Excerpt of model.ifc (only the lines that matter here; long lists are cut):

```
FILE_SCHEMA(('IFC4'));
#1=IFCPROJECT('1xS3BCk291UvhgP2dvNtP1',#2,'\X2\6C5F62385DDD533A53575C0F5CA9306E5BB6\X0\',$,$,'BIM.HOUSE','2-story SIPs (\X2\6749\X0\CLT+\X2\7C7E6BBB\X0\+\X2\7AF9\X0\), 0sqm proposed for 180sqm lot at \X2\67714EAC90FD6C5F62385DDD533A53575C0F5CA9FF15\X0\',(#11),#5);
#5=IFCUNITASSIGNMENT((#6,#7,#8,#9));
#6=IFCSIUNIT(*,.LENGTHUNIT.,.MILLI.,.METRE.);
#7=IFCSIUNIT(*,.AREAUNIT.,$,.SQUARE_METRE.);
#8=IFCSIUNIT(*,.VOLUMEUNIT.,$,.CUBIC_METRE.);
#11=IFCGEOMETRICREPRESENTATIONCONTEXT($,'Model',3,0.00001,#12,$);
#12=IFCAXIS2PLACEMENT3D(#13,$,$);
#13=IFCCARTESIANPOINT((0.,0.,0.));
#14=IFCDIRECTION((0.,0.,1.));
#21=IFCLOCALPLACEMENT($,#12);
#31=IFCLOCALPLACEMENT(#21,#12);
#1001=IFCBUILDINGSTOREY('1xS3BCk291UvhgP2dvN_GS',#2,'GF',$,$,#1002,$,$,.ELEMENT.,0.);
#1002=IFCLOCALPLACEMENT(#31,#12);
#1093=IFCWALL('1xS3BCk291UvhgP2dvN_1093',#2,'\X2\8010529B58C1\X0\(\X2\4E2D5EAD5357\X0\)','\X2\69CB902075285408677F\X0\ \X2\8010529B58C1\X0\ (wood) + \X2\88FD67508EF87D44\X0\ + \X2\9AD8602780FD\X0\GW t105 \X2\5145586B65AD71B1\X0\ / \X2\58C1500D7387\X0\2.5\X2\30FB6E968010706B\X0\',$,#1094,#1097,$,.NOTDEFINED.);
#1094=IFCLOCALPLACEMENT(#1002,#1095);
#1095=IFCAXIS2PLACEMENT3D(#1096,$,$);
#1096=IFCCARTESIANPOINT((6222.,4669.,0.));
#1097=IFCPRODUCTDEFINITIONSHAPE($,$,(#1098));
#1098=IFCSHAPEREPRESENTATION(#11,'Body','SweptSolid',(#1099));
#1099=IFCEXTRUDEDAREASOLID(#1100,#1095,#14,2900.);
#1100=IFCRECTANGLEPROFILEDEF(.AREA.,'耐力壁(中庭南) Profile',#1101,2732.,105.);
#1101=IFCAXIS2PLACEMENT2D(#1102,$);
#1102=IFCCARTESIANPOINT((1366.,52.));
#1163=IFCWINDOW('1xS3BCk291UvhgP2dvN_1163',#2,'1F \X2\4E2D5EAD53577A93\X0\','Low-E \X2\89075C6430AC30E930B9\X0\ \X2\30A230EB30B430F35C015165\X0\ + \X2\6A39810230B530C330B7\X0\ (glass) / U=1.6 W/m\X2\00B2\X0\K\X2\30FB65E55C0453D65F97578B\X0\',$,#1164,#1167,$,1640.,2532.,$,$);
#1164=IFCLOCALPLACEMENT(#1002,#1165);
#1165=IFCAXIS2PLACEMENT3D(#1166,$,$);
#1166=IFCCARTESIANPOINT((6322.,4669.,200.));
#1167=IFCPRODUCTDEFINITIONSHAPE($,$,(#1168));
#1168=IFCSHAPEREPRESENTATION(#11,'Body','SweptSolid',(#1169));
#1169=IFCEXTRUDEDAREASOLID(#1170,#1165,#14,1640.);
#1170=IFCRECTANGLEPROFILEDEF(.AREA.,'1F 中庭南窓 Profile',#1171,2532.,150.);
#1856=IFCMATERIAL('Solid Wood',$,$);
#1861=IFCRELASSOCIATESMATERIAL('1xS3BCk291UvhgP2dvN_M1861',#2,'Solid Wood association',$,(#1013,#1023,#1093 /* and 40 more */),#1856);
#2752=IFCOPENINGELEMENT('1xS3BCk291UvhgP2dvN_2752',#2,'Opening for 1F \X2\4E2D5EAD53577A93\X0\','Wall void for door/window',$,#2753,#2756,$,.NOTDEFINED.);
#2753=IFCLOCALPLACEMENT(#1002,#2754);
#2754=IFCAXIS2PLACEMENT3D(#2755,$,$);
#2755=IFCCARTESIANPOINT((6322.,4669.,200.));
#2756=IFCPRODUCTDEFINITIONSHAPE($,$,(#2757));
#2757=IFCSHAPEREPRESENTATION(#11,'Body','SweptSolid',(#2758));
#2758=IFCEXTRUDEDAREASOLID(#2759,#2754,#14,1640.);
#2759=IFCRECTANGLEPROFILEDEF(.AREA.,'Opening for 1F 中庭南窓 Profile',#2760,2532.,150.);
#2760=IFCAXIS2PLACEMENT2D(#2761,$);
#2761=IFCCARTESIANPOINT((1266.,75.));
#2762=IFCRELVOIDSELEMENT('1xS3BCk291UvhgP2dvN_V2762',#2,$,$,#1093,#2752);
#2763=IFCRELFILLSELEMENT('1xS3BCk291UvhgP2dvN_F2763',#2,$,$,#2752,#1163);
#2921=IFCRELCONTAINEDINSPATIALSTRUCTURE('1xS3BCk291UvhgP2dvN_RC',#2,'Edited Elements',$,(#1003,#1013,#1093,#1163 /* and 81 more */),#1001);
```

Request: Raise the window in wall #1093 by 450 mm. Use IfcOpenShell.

```python
import numpy as np
import ifcopenshell
import ifcopenshell.api.geometry
import ifcopenshell.util.placement
import ifcopenshell.util.unit

model = ifcopenshell.open("model.ifc")
unit_scale = ifcopenshell.util.unit.calculate_unit_scale(model)

window = model.by_id(1163)
opening = window.FillsVoids[0].RelatingOpeningElement
dz = 0.45 / unit_scale

shift = np.array([0.0, 0.0, dz])
# The window is not placed relative to its opening, so move both.
for product in (opening, window):
    matrix = ifcopenshell.util.placement.get_local_placement(product.ObjectPlacement)
    matrix[:3, 3] += shift
    ifcopenshell.api.geometry.edit_object_placement(model, product=product, matrix=matrix, is_si=False)

print(f"moved by {dz * unit_scale:+.3f} m")

model.write("model_updated.ifc")
```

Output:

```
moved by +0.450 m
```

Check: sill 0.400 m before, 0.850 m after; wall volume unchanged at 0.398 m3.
